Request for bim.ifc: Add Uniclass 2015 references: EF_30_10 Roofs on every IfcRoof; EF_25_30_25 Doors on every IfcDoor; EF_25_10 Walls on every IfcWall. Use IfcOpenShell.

First a look at what the model holds.

```python
import ifcopenshell

model = ifcopenshell.open("bim.ifc")
print(model.schema)
print("classifications:", [c.Name for c in model.by_type("IfcClassification")])
for ifc_class in ("IfcDoor", "IfcRoof", "IfcStair", "IfcWall", "IfcWindow"):
    print(ifc_class, len(model.by_type(ifc_class)))
```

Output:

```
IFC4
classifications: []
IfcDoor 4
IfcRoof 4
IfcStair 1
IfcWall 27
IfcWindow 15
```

```python
import ifcopenshell
import ifcopenshell.api.classification

model = ifcopenshell.open("bim.ifc")

system = ifcopenshell.api.classification.add_classification(model, classification="Uniclass 2015")

codes = {
    "IfcRoof": ("EF_30_10", "Roofs"),
    "IfcDoor": ("EF_25_30_25", "Doors"),
    "IfcWall": ("EF_25_10", "Walls"),
}
for ifc_class, (code, name) in codes.items():
    products = model.by_type(ifc_class)
    ifcopenshell.api.classification.add_reference(
        model, products=products, classification=system, identification=code, name=name
    )
    print(code, len(products))

model.write("bim_v2.ifc")
```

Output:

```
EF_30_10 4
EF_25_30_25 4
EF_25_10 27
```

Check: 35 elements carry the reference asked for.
